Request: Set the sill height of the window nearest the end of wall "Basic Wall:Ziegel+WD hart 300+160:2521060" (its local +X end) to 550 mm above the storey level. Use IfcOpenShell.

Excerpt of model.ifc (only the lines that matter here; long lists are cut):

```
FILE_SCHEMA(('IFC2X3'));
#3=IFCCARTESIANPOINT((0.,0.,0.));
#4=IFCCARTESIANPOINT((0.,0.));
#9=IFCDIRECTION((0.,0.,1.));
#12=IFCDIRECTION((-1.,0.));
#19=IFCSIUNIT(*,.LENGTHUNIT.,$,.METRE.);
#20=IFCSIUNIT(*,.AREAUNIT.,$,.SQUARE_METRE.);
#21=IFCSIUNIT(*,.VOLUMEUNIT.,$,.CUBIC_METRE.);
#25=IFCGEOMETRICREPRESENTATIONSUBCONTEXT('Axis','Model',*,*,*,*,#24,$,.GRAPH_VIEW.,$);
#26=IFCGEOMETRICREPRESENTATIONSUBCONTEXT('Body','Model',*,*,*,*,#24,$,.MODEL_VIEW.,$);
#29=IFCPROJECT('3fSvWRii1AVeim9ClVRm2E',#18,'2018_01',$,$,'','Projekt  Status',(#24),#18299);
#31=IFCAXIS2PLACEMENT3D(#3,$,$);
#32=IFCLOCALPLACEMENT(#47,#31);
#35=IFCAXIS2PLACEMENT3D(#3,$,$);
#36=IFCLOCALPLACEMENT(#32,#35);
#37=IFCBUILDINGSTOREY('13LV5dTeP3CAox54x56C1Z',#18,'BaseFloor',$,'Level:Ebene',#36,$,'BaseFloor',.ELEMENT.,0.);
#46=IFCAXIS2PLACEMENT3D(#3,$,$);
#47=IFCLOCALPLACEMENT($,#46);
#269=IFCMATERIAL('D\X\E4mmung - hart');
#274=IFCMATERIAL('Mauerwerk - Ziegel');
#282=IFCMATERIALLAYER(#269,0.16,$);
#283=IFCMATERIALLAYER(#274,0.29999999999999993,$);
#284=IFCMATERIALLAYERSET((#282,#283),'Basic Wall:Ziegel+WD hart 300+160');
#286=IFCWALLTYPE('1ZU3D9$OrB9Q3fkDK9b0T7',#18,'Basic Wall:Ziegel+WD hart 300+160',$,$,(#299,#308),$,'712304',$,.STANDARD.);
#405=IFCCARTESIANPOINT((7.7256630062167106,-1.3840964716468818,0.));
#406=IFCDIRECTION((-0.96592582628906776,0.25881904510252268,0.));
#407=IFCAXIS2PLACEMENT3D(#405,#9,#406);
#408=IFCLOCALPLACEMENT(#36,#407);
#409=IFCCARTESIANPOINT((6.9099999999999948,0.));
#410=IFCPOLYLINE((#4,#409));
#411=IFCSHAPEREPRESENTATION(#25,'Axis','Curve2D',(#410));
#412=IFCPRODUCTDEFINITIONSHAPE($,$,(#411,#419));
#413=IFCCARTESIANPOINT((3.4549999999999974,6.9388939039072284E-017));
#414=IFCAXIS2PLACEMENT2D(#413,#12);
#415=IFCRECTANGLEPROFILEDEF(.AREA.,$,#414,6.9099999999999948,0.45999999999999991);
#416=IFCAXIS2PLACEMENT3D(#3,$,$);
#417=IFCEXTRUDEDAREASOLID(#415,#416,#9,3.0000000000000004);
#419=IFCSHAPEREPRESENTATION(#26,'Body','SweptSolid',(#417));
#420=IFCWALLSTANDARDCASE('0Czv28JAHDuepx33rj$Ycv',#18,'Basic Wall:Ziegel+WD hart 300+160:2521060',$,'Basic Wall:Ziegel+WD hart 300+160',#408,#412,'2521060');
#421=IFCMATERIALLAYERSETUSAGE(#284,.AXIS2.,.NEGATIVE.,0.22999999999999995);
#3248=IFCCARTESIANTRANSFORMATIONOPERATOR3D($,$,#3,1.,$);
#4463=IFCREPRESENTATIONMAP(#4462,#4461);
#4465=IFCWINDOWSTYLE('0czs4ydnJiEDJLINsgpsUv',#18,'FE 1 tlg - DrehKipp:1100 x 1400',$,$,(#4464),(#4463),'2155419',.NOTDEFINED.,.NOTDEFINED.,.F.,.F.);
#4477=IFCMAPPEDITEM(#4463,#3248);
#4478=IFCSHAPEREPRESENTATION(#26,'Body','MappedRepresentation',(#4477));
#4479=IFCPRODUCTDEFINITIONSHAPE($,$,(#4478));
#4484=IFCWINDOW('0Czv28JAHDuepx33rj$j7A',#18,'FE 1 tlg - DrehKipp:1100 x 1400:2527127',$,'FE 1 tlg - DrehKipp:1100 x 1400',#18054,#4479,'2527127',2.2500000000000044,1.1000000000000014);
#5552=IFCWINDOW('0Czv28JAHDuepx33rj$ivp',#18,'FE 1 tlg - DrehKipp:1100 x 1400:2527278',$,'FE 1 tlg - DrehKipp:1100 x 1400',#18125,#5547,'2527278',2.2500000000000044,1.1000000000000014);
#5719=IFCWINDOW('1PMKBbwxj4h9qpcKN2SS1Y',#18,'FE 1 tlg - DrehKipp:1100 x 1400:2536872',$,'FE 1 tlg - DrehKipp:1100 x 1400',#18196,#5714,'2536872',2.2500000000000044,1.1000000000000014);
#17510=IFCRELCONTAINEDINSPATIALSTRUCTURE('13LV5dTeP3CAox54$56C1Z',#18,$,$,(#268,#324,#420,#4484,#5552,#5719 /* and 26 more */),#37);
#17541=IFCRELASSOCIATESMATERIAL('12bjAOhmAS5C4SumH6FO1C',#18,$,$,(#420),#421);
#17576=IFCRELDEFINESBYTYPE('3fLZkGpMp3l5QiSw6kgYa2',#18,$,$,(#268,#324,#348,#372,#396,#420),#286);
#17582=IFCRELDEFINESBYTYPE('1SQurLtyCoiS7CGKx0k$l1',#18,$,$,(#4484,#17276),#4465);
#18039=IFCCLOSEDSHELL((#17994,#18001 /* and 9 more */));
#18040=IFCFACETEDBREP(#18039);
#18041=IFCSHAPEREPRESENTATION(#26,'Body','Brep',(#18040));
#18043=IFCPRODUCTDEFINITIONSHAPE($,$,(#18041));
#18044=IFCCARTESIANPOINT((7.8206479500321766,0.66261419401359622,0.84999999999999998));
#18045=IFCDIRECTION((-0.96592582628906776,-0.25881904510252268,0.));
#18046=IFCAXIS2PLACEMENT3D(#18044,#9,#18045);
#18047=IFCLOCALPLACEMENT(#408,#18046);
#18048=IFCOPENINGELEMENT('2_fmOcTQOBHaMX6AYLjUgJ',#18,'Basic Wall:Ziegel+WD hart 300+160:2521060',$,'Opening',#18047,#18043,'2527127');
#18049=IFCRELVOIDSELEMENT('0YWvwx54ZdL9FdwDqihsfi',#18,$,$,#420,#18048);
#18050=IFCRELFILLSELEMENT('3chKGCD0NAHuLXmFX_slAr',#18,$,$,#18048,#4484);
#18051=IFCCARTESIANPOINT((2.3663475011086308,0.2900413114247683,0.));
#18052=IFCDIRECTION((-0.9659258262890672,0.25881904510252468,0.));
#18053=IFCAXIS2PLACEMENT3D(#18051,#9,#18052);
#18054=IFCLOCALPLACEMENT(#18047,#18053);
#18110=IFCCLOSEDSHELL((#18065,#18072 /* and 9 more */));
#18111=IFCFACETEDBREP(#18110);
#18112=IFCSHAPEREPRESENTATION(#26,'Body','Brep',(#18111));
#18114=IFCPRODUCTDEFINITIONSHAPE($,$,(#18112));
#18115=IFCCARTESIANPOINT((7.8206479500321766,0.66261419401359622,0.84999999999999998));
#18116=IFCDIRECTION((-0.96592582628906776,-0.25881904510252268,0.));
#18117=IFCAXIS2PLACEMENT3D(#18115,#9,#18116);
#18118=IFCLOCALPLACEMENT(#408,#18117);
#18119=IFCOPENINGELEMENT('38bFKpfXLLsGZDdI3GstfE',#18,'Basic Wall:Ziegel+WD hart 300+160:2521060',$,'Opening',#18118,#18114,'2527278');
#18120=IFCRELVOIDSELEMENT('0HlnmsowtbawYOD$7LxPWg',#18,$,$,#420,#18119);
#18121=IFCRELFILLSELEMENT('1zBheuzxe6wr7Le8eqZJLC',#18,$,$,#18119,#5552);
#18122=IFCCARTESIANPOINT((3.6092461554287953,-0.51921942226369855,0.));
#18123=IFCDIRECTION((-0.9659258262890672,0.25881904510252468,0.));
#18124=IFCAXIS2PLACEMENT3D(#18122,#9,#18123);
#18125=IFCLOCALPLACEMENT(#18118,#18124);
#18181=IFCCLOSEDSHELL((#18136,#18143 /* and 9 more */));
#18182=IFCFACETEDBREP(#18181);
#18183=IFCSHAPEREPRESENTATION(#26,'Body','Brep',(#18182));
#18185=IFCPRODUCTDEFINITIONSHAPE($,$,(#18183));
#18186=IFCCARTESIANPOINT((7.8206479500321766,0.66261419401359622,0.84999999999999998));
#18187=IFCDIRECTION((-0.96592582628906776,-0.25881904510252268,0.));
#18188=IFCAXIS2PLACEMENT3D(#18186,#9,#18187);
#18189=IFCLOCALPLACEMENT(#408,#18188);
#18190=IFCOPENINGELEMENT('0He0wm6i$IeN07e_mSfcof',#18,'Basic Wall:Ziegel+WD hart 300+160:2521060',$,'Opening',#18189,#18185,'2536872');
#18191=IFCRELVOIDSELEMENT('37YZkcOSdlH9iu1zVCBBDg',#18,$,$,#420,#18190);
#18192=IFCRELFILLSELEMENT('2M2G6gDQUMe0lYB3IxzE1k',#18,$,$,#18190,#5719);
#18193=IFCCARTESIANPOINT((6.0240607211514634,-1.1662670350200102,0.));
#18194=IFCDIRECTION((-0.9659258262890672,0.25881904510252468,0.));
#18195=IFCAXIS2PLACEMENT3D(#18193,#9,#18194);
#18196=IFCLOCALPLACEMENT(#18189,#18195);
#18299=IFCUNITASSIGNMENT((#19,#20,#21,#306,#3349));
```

```python
import numpy as np
import ifcopenshell
import ifcopenshell.api.geometry
import ifcopenshell.geom
import ifcopenshell.util.element
import ifcopenshell.util.placement
import ifcopenshell.util.shape
import ifcopenshell.util.unit

model = ifcopenshell.open("model.ifc")
unit_scale = ifcopenshell.util.unit.calculate_unit_scale(model)

window = model.by_guid("0Czv28JAHDuepx33rj$j7A")
opening = window.FillsVoids[0].RelatingOpeningElement
storey = ifcopenshell.util.element.get_container(window, ifc_class="IfcBuildingStorey")
level = ifcopenshell.util.placement.get_local_placement(storey.ObjectPlacement)[2, 3]

# The opening's origin need not be at the sill, so measure its lowest point.
shape = ifcopenshell.geom.create_shape(ifcopenshell.geom.settings(), opening)
bottom = ifcopenshell.util.shape.get_shape_bottom_elevation(shape, shape.geometry) / unit_scale
dz = level + 0.55 / unit_scale - bottom

shift = np.array([0.0, 0.0, dz])
# The window is placed relative to its opening, so it follows when the opening moves.
matrix = ifcopenshell.util.placement.get_local_placement(opening.ObjectPlacement)
matrix[:3, 3] += shift
ifcopenshell.api.geometry.edit_object_placement(
    model, product=opening, matrix=matrix, is_si=False, should_transform_children=True
)

print(f"moved by {dz * unit_scale:+.3f} m")

model.write("model-out.ifc")
```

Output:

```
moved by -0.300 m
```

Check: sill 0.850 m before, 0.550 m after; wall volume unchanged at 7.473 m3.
